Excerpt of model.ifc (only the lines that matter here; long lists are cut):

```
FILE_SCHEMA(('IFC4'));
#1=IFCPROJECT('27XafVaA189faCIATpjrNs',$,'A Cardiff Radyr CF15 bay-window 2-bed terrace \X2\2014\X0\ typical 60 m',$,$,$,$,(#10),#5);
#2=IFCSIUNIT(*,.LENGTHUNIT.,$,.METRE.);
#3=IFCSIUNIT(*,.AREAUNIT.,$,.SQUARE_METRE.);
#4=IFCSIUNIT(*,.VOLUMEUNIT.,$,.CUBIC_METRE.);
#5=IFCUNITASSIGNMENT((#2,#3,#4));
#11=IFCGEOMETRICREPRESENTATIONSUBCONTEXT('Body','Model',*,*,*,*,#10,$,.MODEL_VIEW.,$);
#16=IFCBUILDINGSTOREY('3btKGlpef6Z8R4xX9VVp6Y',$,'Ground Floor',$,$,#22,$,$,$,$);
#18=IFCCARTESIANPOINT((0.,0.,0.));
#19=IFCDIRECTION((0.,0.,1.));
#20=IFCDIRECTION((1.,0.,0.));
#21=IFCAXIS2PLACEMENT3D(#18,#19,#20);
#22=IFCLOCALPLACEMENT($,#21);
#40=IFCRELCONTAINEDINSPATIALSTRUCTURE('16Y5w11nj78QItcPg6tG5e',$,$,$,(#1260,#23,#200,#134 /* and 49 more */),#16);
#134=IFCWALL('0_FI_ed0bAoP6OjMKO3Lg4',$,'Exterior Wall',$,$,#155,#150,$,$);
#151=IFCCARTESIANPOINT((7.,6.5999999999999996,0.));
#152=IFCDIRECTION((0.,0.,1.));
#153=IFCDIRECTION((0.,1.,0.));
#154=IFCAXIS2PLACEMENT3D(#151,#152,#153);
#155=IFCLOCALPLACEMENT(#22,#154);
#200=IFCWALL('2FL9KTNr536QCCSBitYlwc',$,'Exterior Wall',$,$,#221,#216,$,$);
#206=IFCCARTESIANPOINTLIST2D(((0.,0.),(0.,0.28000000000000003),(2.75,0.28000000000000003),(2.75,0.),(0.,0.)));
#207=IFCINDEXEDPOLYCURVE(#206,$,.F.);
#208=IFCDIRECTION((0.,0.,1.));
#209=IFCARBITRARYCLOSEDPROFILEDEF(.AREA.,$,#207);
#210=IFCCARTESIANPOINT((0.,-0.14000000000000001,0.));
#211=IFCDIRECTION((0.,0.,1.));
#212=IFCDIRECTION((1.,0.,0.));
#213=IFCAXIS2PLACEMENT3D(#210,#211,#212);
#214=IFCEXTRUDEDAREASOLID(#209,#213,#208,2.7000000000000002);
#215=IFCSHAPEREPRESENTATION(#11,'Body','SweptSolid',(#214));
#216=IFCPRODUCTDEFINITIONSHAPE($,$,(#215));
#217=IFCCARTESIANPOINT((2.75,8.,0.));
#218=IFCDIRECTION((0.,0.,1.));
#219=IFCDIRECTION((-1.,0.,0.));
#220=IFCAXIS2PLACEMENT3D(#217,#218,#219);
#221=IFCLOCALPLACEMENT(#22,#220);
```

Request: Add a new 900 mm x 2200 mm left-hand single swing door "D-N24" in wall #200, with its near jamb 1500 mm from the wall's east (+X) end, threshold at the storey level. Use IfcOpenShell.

```python
import numpy as np
import ifcopenshell
import ifcopenshell.api.feature
import ifcopenshell.api.geometry
import ifcopenshell.api.root
import ifcopenshell.api.spatial
import ifcopenshell.geom
import ifcopenshell.util.element
import ifcopenshell.util.placement
import ifcopenshell.util.representation
import ifcopenshell.util.shape
import ifcopenshell.util.unit

model = ifcopenshell.open("model.ifc")
unit_scale = ifcopenshell.util.unit.calculate_unit_scale(model)
settings = ifcopenshell.geom.settings()


def volume(element):
    """Net volume in cubic metres, openings subtracted."""
    shape = ifcopenshell.geom.create_shape(settings, element)
    return ifcopenshell.util.shape.get_volume(shape.geometry)


wall = model.by_guid("2FL9KTNr536QCCSBitYlwc")
storey = ifcopenshell.util.element.get_container(wall, ifc_class="IfcBuildingStorey")
context = ifcopenshell.util.representation.get_context(model, "Model", "Body", "MODEL_VIEW")
before = volume(wall)

width, height, from_end, sill = 0.9, 2.2, 1.5, 0.0  # metres

# The wall runs along its own X axis, and the end named is its -X end.
wall_shape = ifcopenshell.geom.create_shape(settings, wall)
x, y, z = ifcopenshell.util.shape.get_vertices(wall_shape.geometry).T
start = x.min() + from_end
face, thickness = float(y.min()), float(y.max() - y.min())
wall_matrix = ifcopenshell.util.placement.get_local_placement(wall.ObjectPlacement)
level = ifcopenshell.util.placement.get_local_placement(storey.ObjectPlacement)[2, 3]


def in_wall(x, y):
    """Placement at x, y metres in the wall's axes, at sill height."""
    matrix = wall_matrix.copy()
    matrix[:, 3] = wall_matrix @ np.array([x / unit_scale, y / unit_scale, 0.0, 1.0])
    matrix[2, 3] = level + sill / unit_scale
    return matrix


# Opening: a box that overshoots both wall faces by 50 mm.
opening = ifcopenshell.api.root.create_entity(model, ifc_class="IfcOpeningElement", predefined_type="OPENING")
box = ifcopenshell.api.geometry.add_wall_representation(
    model, context=context, length=width, height=height, thickness=thickness + 0.1
)
ifcopenshell.api.geometry.assign_representation(model, product=opening, representation=box)
ifcopenshell.api.geometry.edit_object_placement(model, product=opening, matrix=in_wall(start, face - 0.05), is_si=False)
ifcopenshell.api.feature.add_feature(model, feature=opening, element=wall)

door = ifcopenshell.api.root.create_entity(model, ifc_class="IfcDoor", name="D-N24", predefined_type="DOOR")
door.OverallWidth, door.OverallHeight = width / unit_scale, height / unit_scale
door.OperationType = "SINGLE_SWING_LEFT"
body = ifcopenshell.api.geometry.add_door_representation(
    model,
    context=context,
    overall_width=door.OverallWidth,
    overall_height=door.OverallHeight,
    operation_type="SINGLE_SWING_LEFT",
    lining_properties={"LiningDepth": thickness / unit_scale, "ThresholdDepth": thickness / unit_scale},
)
ifcopenshell.api.geometry.assign_representation(model, product=door, representation=body)
ifcopenshell.api.spatial.assign_container(model, products=[door], relating_structure=storey)
ifcopenshell.api.feature.add_filling(model, opening=opening, element=door)

# The lining spans the wall, so the door starts at the wall face.
ifcopenshell.api.geometry.edit_object_placement(model, product=door, matrix=in_wall(start, face), is_si=False)

after = volume(wall)

print(f"wall volume {before:.3f} -> {after:.3f} m3")

model.write("model_updated.ifc")
```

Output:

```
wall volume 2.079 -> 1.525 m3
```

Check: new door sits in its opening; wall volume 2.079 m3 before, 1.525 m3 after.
